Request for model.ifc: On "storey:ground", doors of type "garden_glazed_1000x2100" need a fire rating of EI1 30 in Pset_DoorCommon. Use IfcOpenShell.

First a look at what the model holds.

```python
import ifcopenshell
import ifcopenshell.util.element

model = ifcopenshell.open("model.ifc")
print(model.schema)
storey = next(s for s in model.by_type("IfcBuildingStorey") if s.Name == "storey:ground")
doors = [e for e in ifcopenshell.util.element.get_decomposition(storey) if e.is_a("IfcDoor")]
seen = {}
for e in doors:
    element_type = ifcopenshell.util.element.get_type(e)
    key = (element_type.Name if element_type != e and element_type else None, ifcopenshell.util.element.get_pset(e, "Pset_DoorCommon", "FireRating"))
    seen[key] = seen.get(key, 0) + 1
for (name, value), count in sorted(seen.items(), key=str):
    print(count, "x", name, "|", value)
```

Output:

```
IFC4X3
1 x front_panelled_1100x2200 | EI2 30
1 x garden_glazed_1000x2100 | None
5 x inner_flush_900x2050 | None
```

```python
import ifcopenshell
import ifcopenshell.api.pset
import ifcopenshell.util.element

model = ifcopenshell.open("model.ifc")

storey = next(s for s in model.by_type("IfcBuildingStorey") if s.Name == "storey:ground")
doors = [e for e in ifcopenshell.util.element.get_decomposition(storey) if e.is_a("IfcDoor")]

count = 0
for e in doors:
    element_type = ifcopenshell.util.element.get_type(e)
    if element_type in (None, e) or element_type.Name != "garden_glazed_1000x2100":
        continue
    # add_pset returns the element's existing set when there is one.
    pset = ifcopenshell.api.pset.add_pset(model, product=e, name="Pset_DoorCommon")
    ifcopenshell.api.pset.edit_pset(model, pset=pset, properties={"FireRating": "EI1 30"})
    count += 1

print(count, "doors updated")

model.write("model_rev.ifc")
```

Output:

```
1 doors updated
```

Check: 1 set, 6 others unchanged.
